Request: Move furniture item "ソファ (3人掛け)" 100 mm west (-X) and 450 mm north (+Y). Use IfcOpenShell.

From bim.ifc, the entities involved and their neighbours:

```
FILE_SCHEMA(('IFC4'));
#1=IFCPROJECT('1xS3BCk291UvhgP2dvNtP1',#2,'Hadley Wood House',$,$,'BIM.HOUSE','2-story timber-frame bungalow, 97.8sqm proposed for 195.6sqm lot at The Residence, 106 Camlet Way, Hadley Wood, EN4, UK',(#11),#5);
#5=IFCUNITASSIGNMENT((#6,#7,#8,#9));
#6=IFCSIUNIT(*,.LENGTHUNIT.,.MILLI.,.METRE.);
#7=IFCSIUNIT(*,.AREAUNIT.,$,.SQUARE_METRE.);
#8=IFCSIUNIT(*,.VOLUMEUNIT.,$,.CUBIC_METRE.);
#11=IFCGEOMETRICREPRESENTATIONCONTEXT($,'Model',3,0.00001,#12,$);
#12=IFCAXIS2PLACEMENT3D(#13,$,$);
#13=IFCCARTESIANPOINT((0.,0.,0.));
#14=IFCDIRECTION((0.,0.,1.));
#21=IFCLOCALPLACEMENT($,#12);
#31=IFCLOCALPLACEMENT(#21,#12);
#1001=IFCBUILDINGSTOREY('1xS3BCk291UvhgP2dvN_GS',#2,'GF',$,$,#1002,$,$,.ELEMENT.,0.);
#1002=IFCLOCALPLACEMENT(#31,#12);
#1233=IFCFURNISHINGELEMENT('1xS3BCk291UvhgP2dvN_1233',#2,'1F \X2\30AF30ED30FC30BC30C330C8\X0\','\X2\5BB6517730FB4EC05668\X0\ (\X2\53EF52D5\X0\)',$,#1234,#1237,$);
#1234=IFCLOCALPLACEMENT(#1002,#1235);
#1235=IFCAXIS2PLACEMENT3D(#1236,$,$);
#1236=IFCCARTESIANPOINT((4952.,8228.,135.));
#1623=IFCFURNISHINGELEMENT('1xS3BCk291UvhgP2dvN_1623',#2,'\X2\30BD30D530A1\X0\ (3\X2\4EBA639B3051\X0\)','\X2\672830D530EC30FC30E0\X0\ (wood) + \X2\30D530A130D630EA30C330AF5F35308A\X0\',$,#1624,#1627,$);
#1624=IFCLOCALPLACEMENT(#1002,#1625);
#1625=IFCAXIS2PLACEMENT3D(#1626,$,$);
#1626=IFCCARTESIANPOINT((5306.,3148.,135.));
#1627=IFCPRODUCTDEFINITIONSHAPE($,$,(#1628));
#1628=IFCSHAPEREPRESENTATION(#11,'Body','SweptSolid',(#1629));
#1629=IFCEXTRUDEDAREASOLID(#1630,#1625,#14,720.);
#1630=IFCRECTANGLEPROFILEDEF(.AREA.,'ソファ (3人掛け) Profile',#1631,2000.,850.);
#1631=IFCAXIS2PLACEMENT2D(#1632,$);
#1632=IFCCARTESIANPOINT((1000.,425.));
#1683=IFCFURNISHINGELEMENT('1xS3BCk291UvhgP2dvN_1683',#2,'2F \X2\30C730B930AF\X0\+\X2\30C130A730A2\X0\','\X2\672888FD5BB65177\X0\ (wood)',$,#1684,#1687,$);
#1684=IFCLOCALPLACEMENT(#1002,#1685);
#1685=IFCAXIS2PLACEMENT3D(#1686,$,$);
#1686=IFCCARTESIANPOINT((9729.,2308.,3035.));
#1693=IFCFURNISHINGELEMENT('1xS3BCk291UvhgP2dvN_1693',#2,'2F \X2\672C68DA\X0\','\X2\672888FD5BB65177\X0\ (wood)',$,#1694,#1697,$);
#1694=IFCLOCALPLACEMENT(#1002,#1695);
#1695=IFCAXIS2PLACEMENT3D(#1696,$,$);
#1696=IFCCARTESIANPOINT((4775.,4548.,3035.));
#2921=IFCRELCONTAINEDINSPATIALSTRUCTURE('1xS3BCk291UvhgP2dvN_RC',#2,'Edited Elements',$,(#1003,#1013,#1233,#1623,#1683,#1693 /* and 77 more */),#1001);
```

```python
import ifcopenshell
import ifcopenshell.api.geometry
import ifcopenshell.util.placement
import ifcopenshell.util.unit

model = ifcopenshell.open("bim.ifc")
unit_scale = ifcopenshell.util.unit.calculate_unit_scale(model)

item = model.by_id(1623)
matrix = ifcopenshell.util.placement.get_local_placement(item.ObjectPlacement)
matrix[0, 3] -= 0.1 / unit_scale
matrix[1, 3] += 0.45 / unit_scale
ifcopenshell.api.geometry.edit_object_placement(model, product=item, matrix=matrix, is_si=False)

print(ifcopenshell.util.placement.get_local_placement(item.ObjectPlacement).round(3) + 0.0)

model.write("bim_v2.ifc")
```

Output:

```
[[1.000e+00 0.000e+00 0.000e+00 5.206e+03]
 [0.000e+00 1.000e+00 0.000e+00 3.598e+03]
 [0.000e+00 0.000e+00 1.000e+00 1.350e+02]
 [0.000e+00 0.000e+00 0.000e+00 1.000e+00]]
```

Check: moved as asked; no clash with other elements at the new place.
